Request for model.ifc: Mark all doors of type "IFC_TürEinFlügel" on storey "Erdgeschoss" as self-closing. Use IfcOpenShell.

First a look at what the model holds.

```python
import ifcopenshell
import ifcopenshell.util.element

model = ifcopenshell.open("model.ifc")
print(model.schema)
storey = next(s for s in model.by_type("IfcBuildingStorey") if s.Name == "Erdgeschoss")
doors = [e for e in ifcopenshell.util.element.get_decomposition(storey) if e.is_a("IfcDoor")]
seen = {}
for e in doors:
    element_type = ifcopenshell.util.element.get_type(e)
    key = (element_type.Name if element_type != e and element_type else None, ifcopenshell.util.element.get_pset(e, "Pset_DoorCommon", "SelfClosing"))
    seen[key] = seen.get(key, 0) + 1
for (name, value), count in sorted(seen.items(), key=str):
    print(count, "x", name, "|", value)
```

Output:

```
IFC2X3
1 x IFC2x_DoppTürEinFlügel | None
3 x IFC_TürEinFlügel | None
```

```python
import ifcopenshell
import ifcopenshell.api.pset
import ifcopenshell.util.element

model = ifcopenshell.open("model.ifc")

storey = next(s for s in model.by_type("IfcBuildingStorey") if s.Name == "Erdgeschoss")
doors = [e for e in ifcopenshell.util.element.get_decomposition(storey) if e.is_a("IfcDoor")]

count = 0
for e in doors:
    element_type = ifcopenshell.util.element.get_type(e)
    if element_type in (None, e) or element_type.Name != "IFC_TürEinFlügel":
        continue
    # add_pset returns the element's existing set when there is one.
    pset = ifcopenshell.api.pset.add_pset(model, product=e, name="Pset_DoorCommon")
    ifcopenshell.api.pset.edit_pset(model, pset=pset, properties={"SelfClosing": True})
    count += 1

print(count, "doors updated")

model.write("model_rev.ifc")
```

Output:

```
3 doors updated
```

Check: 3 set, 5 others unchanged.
